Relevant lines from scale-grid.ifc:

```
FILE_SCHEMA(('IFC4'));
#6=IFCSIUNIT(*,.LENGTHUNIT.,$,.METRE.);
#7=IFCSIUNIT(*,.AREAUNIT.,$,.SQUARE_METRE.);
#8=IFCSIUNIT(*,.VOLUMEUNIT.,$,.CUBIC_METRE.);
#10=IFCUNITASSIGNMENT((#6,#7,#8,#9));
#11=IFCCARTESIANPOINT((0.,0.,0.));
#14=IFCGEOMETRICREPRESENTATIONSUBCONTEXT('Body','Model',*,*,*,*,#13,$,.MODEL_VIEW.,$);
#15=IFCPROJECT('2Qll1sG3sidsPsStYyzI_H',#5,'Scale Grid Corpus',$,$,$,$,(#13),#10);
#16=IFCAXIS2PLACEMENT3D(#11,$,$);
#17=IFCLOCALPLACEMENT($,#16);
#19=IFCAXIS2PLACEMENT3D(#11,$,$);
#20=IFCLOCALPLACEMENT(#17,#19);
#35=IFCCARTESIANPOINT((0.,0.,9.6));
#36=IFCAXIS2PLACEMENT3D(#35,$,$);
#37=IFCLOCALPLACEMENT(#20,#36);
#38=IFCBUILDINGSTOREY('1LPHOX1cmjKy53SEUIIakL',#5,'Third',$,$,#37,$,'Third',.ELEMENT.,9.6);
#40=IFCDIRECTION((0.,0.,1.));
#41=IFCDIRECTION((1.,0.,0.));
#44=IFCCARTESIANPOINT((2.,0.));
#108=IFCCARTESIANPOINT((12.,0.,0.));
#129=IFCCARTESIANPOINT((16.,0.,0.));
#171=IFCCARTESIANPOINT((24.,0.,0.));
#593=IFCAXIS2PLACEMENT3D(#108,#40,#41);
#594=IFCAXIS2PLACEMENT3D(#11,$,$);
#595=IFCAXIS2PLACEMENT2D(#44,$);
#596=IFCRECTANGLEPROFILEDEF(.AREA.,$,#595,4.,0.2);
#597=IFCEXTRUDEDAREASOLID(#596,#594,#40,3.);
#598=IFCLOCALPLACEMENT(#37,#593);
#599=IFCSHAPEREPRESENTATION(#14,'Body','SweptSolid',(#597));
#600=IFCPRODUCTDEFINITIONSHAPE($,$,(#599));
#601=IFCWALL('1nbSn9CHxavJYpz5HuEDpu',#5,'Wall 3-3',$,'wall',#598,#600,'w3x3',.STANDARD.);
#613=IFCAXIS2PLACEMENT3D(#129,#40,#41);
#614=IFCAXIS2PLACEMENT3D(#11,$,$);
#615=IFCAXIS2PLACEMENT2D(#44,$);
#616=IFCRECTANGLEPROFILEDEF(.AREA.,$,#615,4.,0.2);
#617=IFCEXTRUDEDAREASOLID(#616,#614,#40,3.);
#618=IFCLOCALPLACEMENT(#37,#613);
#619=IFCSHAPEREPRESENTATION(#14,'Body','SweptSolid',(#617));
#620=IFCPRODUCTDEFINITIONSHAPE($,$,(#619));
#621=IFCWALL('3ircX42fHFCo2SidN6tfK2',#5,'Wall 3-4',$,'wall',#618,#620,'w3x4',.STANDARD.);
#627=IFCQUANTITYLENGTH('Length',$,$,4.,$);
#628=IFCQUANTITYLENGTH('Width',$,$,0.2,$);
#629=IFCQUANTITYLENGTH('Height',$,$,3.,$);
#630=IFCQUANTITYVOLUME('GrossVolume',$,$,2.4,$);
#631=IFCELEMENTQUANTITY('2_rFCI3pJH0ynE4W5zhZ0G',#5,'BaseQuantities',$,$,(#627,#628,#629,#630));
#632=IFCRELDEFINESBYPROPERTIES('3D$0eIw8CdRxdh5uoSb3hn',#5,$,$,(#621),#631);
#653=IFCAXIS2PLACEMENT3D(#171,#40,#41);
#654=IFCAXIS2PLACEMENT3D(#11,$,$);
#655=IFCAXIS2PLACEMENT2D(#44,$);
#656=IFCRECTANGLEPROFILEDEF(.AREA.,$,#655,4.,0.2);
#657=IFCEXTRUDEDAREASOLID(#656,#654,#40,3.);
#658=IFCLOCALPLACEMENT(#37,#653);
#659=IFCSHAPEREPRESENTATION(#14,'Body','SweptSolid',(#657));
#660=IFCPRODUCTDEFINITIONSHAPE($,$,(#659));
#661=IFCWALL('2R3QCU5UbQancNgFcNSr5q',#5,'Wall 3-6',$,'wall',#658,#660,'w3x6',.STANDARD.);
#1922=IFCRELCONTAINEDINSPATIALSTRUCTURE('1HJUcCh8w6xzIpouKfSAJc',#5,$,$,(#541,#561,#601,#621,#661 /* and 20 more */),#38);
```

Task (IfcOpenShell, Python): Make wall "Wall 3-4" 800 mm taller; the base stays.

```python
import ifcopenshell
import ifcopenshell.api.pset
import ifcopenshell.geom
import ifcopenshell.util.element
import ifcopenshell.util.representation
import ifcopenshell.util.shape
import ifcopenshell.util.unit

model = ifcopenshell.open("scale-grid.ifc")
unit_scale = ifcopenshell.util.unit.calculate_unit_scale(model)
volume_scale = ifcopenshell.util.unit.calculate_unit_scale(model, "VOLUMEUNIT")
settings = ifcopenshell.geom.settings()


def volume(element):
    """Net volume in cubic metres, openings subtracted."""
    shape = ifcopenshell.geom.create_shape(settings, element)
    return ifcopenshell.util.shape.get_volume(shape.geometry)


wall = model.by_id(621)
before = volume(wall)

body = ifcopenshell.util.representation.get_representation(wall, "Model", "Body")
solid = body.Items[0]
old_height = solid.Depth
solid.Depth += 0.8 / unit_scale
after = volume(wall)

# Update the stored height, areas and volumes.
qto = model.by_id(ifcopenshell.util.element.get_pset(wall, "BaseQuantities", should_inherit=False)["id"])
ifcopenshell.api.pset.edit_qto(model, qto=qto, properties={
    "Height": solid.Depth,
    "GrossVolume": ifcopenshell.util.element.get_pset(wall, "BaseQuantities", "GrossVolume") * solid.Depth / old_height,
})

print(f"height {old_height:g} -> {solid.Depth:g}, volume {before:.3f} -> {after:.3f} m3")

model.write("scale-grid_rev.ifc")
```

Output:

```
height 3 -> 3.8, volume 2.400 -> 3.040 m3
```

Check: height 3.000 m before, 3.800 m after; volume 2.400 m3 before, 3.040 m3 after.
